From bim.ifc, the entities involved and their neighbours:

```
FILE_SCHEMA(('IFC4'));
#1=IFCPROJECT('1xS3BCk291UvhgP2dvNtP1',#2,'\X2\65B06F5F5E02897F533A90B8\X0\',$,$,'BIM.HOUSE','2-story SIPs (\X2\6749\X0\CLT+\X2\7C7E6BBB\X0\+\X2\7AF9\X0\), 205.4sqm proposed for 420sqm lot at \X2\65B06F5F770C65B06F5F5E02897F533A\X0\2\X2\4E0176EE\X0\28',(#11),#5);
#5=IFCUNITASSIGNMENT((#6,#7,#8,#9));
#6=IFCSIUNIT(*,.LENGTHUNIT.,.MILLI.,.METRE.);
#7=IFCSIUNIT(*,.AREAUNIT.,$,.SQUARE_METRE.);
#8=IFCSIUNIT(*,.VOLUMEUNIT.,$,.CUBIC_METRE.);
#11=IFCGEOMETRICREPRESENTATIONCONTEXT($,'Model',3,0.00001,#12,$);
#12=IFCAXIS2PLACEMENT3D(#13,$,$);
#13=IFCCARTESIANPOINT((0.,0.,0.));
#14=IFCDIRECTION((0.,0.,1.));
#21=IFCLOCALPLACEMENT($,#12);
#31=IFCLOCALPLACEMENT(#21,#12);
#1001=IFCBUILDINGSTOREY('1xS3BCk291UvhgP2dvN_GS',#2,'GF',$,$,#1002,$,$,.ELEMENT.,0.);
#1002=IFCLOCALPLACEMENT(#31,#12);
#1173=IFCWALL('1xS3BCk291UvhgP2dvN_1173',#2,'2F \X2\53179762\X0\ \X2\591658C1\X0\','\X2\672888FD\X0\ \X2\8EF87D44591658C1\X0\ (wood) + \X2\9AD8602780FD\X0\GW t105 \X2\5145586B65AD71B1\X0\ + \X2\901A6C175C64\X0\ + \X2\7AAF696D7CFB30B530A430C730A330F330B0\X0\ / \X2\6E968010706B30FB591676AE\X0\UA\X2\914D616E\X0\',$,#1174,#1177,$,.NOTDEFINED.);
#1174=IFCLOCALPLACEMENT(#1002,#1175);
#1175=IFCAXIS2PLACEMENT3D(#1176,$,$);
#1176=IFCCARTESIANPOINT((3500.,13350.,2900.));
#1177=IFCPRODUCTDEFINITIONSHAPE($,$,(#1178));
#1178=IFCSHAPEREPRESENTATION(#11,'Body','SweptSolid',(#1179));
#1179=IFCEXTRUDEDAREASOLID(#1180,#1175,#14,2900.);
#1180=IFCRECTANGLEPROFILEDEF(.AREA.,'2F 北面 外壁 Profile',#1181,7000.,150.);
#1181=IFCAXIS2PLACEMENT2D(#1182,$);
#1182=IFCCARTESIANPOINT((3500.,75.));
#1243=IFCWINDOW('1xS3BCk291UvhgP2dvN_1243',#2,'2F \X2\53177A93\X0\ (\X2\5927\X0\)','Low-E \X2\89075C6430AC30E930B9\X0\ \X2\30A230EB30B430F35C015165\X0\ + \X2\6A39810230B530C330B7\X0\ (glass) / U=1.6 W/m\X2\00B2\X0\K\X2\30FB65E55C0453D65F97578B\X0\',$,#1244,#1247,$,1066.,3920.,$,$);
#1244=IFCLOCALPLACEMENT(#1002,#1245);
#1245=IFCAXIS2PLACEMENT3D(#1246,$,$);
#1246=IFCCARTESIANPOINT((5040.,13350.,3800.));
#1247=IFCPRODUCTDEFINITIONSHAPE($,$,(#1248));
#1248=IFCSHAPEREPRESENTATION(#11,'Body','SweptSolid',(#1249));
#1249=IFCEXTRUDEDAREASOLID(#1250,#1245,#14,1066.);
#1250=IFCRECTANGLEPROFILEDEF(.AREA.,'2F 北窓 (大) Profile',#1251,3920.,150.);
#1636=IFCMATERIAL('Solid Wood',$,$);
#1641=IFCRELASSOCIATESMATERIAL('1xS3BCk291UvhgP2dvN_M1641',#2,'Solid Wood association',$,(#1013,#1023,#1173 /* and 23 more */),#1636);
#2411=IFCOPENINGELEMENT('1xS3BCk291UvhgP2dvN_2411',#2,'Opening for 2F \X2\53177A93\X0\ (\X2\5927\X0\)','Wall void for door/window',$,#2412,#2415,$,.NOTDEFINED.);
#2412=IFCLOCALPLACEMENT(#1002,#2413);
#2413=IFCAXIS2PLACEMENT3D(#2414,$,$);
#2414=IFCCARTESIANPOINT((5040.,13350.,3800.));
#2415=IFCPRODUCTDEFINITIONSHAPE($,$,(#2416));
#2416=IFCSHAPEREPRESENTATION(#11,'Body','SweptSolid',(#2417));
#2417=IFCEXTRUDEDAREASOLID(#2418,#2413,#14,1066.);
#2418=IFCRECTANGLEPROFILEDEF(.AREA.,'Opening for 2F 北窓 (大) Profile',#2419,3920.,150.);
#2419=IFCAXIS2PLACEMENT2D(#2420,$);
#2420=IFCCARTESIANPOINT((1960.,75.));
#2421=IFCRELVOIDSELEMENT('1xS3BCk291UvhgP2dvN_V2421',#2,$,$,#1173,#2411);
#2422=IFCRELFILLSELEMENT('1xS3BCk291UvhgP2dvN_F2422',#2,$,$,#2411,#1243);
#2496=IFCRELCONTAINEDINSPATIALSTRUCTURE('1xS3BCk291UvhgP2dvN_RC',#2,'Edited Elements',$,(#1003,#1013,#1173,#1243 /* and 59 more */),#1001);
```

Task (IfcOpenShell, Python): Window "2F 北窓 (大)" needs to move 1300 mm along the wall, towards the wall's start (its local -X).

```python
import ifcopenshell
import ifcopenshell.api.geometry
import ifcopenshell.util.placement
import ifcopenshell.util.unit

model = ifcopenshell.open("bim.ifc")
unit_scale = ifcopenshell.util.unit.calculate_unit_scale(model)

window = model.by_guid("1xS3BCk291UvhgP2dvN_1243")
opening = window.FillsVoids[0].RelatingOpeningElement
wall = opening.VoidsElements[0].RelatingBuildingElement

wall_matrix = ifcopenshell.util.placement.get_local_placement(wall.ObjectPlacement)
shift = wall_matrix[:3, 0] * -1.3 / unit_scale
before = ifcopenshell.util.placement.get_local_placement(window.ObjectPlacement)[:3, 3].copy()

# The window is not placed relative to its opening, so move both.
for product in (opening, window):
    matrix = ifcopenshell.util.placement.get_local_placement(product.ObjectPlacement)
    matrix[:3, 3] += shift
    ifcopenshell.api.geometry.edit_object_placement(model, product=product, matrix=matrix, is_si=False)

after = ifcopenshell.util.placement.get_local_placement(window.ObjectPlacement)[:3, 3]
print("window moved by", (after - before).round(3) + 0.0)

model.write("bim-out.ifc")
```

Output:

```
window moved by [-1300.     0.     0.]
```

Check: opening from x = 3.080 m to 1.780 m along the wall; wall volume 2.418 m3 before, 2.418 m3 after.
